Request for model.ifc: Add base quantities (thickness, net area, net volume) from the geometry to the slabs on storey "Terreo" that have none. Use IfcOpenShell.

First a look at what the model holds.

```python
import ifcopenshell
import ifcopenshell.util.element
import ifcopenshell.util.unit

model = ifcopenshell.open("model.ifc")
print(model.schema)
for unit_type in ("LENGTHUNIT", "AREAUNIT", "VOLUMEUNIT"):
    print(unit_type, ifcopenshell.util.unit.calculate_unit_scale(model, unit_type))
storey = next(s for s in model.by_type("IfcBuildingStorey") if s.Name == "Terreo")
slabs = [e for e in ifcopenshell.util.element.get_decomposition(storey) if e.is_a("IfcSlab")]
for e in sorted(slabs, key=lambda e: e.id()):
    print(e.id(), e.is_a(), e.Name, list(ifcopenshell.util.element.get_psets(e, qtos_only=True)), sep=" | ")
```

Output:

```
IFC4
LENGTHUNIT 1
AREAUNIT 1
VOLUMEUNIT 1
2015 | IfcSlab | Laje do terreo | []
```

```python
import ifcopenshell
import ifcopenshell.api.pset
import ifcopenshell.geom
import ifcopenshell.util.element
import ifcopenshell.util.shape
import ifcopenshell.util.unit

model = ifcopenshell.open("model.ifc")
unit_scale = ifcopenshell.util.unit.calculate_unit_scale(model)
area_scale = ifcopenshell.util.unit.calculate_unit_scale(model, "AREAUNIT")
volume_scale = ifcopenshell.util.unit.calculate_unit_scale(model, "VOLUMEUNIT")
settings = ifcopenshell.geom.settings()

storey = next(s for s in model.by_type("IfcBuildingStorey") if s.Name == "Terreo")
slabs = [e for e in ifcopenshell.util.element.get_decomposition(storey) if e.is_a("IfcSlab")]

for e in sorted(slabs, key=lambda e: e.id()):
    if ifcopenshell.util.element.get_psets(e, qtos_only=True, should_inherit=False):
        continue
    # Geometry comes back in metres, in the element's own axes.
    shape = ifcopenshell.geom.create_shape(settings, e)
    values = {
        "Width": ifcopenshell.util.shape.get_z(shape.geometry) / unit_scale,
        "NetArea": ifcopenshell.util.shape.get_footprint_area(shape.geometry) / area_scale,
        "NetVolume": ifcopenshell.util.shape.get_volume(shape.geometry) / volume_scale,
    }
    qto = ifcopenshell.api.pset.add_qto(model, product=e, name="Qto_SlabBaseQuantities")
    ifcopenshell.api.pset.edit_qto(model, qto=qto, properties=values)
    print(e.id(), {k: round(v, 3) for k, v in values.items()})

model.write("model_edited.ifc")
```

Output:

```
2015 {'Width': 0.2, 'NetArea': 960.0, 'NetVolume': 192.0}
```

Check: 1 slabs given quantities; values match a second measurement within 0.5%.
